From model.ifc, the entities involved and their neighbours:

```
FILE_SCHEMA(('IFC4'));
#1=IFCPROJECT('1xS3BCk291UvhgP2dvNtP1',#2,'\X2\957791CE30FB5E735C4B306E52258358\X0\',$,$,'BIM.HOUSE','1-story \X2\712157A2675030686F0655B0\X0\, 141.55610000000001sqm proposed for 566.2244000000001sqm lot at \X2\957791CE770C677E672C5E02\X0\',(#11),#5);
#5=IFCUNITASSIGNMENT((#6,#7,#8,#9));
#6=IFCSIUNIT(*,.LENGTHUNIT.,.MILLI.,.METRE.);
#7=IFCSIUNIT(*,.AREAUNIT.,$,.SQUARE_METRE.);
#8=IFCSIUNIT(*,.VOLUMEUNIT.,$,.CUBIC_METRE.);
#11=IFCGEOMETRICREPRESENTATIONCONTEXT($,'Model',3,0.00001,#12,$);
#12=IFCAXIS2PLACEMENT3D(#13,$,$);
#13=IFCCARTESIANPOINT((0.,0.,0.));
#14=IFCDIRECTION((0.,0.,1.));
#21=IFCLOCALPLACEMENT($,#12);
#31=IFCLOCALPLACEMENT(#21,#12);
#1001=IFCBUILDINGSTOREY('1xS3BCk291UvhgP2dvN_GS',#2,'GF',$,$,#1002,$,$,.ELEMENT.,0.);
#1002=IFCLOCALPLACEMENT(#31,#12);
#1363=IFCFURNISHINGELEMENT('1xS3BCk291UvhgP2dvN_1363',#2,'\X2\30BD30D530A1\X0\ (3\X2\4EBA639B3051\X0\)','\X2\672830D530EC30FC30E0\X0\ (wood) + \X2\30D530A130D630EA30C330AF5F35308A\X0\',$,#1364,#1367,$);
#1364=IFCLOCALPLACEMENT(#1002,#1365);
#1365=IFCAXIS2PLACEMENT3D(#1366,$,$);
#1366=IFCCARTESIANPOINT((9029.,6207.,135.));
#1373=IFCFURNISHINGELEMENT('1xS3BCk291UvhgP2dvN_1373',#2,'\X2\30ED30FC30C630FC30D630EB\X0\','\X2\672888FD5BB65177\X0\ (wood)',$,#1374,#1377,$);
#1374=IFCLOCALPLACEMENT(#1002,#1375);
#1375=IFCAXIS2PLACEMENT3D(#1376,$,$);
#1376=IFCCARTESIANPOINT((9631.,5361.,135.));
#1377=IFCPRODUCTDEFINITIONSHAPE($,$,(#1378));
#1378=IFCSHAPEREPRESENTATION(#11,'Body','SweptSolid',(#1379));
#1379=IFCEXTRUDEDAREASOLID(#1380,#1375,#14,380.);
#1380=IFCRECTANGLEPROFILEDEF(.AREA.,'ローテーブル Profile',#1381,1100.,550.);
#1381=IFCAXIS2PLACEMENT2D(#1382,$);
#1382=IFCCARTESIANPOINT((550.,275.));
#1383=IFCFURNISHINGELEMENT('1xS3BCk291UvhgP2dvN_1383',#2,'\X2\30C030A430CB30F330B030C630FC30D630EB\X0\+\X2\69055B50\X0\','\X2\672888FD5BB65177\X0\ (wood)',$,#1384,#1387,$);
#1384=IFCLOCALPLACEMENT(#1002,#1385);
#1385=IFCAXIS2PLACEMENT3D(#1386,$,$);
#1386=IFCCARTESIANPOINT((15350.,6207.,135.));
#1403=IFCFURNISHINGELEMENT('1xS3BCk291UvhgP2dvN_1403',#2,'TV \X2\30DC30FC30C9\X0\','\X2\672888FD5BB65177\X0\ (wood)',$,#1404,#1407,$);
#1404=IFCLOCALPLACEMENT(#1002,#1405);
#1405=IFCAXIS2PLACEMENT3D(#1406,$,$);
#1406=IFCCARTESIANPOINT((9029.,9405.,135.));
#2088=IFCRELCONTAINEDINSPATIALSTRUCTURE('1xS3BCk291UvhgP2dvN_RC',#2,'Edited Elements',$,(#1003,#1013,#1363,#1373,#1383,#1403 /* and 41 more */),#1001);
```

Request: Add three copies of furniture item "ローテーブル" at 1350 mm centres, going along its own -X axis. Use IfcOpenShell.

```python
import ifcopenshell
import ifcopenshell.api.geometry
import ifcopenshell.api.root
import ifcopenshell.util.element
import ifcopenshell.util.placement
import ifcopenshell.util.unit

model = ifcopenshell.open("model.ifc")
unit_scale = ifcopenshell.util.unit.calculate_unit_scale(model)


def reuse_history(source, copy):
    """copy_class also copies each property set's owner history, people and application; keep the originals."""
    for rel in copy.IsDefinedBy:
        if rel.is_a("IfcRelDefinesByProperties") and (history := rel.RelatingPropertyDefinition.OwnerHistory):
            rel.RelatingPropertyDefinition.OwnerHistory = source.OwnerHistory
            ifcopenshell.util.element.remove_deep2(model, history)


source = model.by_id(1373)
base = ifcopenshell.util.placement.get_local_placement(source.ObjectPlacement)
step = -base[:3, 0] * 1.35 / unit_scale

for i in range(1, 4):
    copy = ifcopenshell.api.root.copy_class(model, product=source)
    copy.Representation = ifcopenshell.util.element.copy_deep(
        model, source.Representation, exclude=["IfcGeometricRepresentationContext", "IfcRepresentationMap"]
    )
    reuse_history(source, copy)
    matrix = base.copy()
    matrix[:3, 3] += i * step
    print("added at", matrix[:3, 3].round(3) + 0.0)
    ifcopenshell.api.geometry.edit_object_placement(model, product=copy, matrix=matrix, is_si=False)

model.write("model_updated.ifc")
```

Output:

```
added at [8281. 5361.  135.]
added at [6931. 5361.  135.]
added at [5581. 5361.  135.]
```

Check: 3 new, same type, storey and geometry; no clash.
